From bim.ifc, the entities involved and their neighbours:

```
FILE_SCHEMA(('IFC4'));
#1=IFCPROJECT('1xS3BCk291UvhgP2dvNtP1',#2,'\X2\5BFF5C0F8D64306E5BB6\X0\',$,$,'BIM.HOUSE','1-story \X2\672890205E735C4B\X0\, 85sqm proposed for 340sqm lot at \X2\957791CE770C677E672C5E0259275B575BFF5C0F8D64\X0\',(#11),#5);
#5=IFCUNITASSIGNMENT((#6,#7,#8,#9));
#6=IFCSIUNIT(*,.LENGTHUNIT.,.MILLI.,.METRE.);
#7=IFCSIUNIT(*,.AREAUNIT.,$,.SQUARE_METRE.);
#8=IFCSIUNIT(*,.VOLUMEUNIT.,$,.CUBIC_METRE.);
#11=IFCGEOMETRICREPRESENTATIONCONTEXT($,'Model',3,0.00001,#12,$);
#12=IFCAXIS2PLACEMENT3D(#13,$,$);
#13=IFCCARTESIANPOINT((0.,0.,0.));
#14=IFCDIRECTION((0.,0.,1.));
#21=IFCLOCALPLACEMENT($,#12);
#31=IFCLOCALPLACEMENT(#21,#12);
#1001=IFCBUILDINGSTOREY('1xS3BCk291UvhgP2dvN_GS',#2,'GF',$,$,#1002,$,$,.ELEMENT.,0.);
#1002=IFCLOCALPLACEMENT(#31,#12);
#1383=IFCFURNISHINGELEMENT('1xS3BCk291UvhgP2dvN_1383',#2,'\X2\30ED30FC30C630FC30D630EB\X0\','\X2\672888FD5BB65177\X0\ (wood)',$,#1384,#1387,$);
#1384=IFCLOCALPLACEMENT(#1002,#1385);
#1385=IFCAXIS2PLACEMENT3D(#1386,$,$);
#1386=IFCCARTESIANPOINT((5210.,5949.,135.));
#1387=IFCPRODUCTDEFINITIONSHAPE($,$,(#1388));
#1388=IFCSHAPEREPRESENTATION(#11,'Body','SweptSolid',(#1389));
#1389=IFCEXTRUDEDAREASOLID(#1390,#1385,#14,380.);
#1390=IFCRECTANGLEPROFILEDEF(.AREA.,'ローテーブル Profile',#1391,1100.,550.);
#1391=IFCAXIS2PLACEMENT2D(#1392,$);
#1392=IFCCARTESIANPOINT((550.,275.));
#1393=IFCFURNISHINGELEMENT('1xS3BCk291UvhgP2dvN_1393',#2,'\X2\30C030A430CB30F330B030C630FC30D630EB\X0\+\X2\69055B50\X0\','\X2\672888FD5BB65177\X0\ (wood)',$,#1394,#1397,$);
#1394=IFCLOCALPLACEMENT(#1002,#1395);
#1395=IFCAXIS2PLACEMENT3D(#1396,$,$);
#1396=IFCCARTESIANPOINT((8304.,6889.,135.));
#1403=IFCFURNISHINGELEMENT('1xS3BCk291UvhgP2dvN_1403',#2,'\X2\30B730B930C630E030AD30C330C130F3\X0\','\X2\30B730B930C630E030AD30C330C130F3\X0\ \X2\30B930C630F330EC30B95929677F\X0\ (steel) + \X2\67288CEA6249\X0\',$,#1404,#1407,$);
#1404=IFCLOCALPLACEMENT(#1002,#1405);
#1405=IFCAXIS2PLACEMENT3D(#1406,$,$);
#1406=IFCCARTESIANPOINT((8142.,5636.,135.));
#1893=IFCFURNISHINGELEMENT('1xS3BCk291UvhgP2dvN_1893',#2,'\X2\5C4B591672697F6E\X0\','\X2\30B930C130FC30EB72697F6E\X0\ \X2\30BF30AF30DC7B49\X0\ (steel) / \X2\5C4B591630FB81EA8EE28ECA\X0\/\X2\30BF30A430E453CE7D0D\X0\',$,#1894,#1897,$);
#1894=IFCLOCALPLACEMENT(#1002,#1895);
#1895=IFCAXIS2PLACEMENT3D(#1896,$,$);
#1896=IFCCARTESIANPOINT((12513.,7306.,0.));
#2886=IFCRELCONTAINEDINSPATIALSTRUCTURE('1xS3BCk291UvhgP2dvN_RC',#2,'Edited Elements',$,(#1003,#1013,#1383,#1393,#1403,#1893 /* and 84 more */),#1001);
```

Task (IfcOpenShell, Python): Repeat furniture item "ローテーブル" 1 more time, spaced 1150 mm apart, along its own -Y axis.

```python
import ifcopenshell
import ifcopenshell.api.geometry
import ifcopenshell.api.root
import ifcopenshell.util.element
import ifcopenshell.util.placement

model = ifcopenshell.open("bim.ifc")


def reuse_history(source, copy):
    """copy_class also copies each property set's owner history, people and application; keep the originals."""
    for rel in copy.IsDefinedBy:
        if rel.is_a("IfcRelDefinesByProperties") and (history := rel.RelatingPropertyDefinition.OwnerHistory):
            rel.RelatingPropertyDefinition.OwnerHistory = source.OwnerHistory
            ifcopenshell.util.element.remove_deep2(model, history)


source = model.by_guid("1xS3BCk291UvhgP2dvN_1383")
base = ifcopenshell.util.placement.get_local_placement(source.ObjectPlacement)
step = -base[:3, 1] * 1150.0

for i in range(1, 2):
    copy = ifcopenshell.api.root.copy_class(model, product=source)
    copy.Representation = ifcopenshell.util.element.copy_deep(
        model, source.Representation, exclude=["IfcGeometricRepresentationContext", "IfcRepresentationMap"]
    )
    reuse_history(source, copy)
    matrix = base.copy()
    matrix[:3, 3] += i * step
    print("added at", matrix[:3, 3].round(3) + 0.0)
    ifcopenshell.api.geometry.edit_object_placement(model, product=copy, matrix=matrix, is_si=False)

model.write("bim_rev.ifc")
```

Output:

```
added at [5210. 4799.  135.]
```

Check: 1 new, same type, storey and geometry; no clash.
